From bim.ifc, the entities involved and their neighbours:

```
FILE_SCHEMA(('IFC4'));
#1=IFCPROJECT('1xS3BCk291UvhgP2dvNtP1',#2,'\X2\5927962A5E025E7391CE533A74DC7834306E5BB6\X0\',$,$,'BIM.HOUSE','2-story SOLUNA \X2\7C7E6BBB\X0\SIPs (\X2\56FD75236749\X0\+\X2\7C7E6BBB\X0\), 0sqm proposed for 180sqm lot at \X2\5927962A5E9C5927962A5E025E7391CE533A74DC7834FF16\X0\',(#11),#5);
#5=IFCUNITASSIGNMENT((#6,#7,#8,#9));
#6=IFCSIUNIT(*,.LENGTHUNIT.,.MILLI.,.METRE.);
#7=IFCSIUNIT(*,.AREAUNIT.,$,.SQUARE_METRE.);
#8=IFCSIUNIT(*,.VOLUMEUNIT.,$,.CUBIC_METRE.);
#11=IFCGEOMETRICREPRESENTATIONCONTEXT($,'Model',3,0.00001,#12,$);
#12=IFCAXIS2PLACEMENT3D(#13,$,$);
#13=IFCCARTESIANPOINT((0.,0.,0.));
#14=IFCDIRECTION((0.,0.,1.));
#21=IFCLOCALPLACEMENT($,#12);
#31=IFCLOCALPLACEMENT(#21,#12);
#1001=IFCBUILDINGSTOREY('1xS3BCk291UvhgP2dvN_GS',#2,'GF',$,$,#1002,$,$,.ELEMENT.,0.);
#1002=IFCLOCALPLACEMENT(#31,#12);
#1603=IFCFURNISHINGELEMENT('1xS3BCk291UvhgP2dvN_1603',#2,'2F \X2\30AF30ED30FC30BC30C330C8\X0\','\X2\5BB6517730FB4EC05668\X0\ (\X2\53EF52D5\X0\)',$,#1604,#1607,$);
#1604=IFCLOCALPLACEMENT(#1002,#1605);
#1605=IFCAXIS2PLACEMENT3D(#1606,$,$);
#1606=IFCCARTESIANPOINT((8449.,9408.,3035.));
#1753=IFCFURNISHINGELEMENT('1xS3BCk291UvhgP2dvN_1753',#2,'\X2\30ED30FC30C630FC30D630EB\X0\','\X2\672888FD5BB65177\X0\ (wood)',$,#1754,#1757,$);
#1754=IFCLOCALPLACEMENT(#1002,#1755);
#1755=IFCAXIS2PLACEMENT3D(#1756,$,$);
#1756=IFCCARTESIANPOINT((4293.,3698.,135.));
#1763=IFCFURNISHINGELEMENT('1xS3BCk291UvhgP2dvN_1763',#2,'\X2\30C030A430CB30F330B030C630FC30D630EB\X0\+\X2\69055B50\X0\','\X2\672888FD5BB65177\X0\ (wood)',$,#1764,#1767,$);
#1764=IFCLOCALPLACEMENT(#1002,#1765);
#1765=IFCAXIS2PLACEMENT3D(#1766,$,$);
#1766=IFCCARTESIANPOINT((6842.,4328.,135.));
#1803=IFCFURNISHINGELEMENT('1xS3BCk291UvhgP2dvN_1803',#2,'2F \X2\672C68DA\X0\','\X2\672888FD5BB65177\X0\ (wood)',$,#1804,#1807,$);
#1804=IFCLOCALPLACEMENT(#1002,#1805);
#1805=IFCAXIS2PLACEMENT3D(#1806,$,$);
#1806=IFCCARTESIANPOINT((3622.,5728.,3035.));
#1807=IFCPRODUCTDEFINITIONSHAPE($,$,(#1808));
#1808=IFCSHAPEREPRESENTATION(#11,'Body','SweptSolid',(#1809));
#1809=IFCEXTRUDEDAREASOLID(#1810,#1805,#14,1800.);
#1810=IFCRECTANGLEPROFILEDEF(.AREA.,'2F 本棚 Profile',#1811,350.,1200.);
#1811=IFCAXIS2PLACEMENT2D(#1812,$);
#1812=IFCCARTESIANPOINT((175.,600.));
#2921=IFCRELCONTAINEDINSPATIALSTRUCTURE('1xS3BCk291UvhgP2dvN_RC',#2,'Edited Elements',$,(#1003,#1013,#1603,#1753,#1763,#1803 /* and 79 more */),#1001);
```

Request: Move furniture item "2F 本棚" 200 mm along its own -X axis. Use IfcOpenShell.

```python
import ifcopenshell
import ifcopenshell.api.geometry
import ifcopenshell.util.placement
import ifcopenshell.util.unit

model = ifcopenshell.open("bim.ifc")
unit_scale = ifcopenshell.util.unit.calculate_unit_scale(model)

item = model.by_id(1803)
matrix = ifcopenshell.util.placement.get_local_placement(item.ObjectPlacement)
matrix[:3, 3] -= matrix[:3, 0] * 0.2 / unit_scale
ifcopenshell.api.geometry.edit_object_placement(model, product=item, matrix=matrix, is_si=False)

print(ifcopenshell.util.placement.get_local_placement(item.ObjectPlacement).round(3) + 0.0)

model.write("bim_updated.ifc")
```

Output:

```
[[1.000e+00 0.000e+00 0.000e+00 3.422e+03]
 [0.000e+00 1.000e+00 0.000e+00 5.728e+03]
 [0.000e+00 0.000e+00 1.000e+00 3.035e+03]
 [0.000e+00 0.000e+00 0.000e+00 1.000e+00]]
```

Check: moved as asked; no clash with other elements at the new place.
